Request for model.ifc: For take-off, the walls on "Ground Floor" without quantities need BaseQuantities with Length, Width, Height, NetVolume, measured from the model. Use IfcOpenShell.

First a look at what the model holds.

```python
import ifcopenshell
import ifcopenshell.util.element
import ifcopenshell.util.unit

model = ifcopenshell.open("model.ifc")
print(model.schema)
for unit_type in ("LENGTHUNIT", "AREAUNIT", "VOLUMEUNIT"):
    print(unit_type, ifcopenshell.util.unit.calculate_unit_scale(model, unit_type))
storey = next(s for s in model.by_type("IfcBuildingStorey") if s.Name == "Ground Floor")
walls = [e for e in ifcopenshell.util.element.get_decomposition(storey) if e.is_a("IfcWall")]
for e in sorted(walls, key=lambda e: e.id()):
    print(e.id(), e.is_a(), e.Name, list(ifcopenshell.util.element.get_psets(e, qtos_only=True)), sep=" | ")
```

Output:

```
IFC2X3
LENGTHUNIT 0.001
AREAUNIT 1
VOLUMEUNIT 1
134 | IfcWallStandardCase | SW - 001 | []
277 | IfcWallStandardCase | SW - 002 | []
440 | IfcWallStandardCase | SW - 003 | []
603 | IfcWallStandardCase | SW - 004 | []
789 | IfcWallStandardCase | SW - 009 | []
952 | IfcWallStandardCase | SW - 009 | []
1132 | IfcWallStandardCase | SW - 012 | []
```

```python
import ifcopenshell
import ifcopenshell.api.pset
import ifcopenshell.geom
import ifcopenshell.util.element
import ifcopenshell.util.shape
import ifcopenshell.util.unit

model = ifcopenshell.open("model.ifc")
unit_scale = ifcopenshell.util.unit.calculate_unit_scale(model)
volume_scale = ifcopenshell.util.unit.calculate_unit_scale(model, "VOLUMEUNIT")
settings = ifcopenshell.geom.settings()

storey = next(s for s in model.by_type("IfcBuildingStorey") if s.Name == "Ground Floor")
walls = [e for e in ifcopenshell.util.element.get_decomposition(storey) if e.is_a("IfcWall")]

for e in sorted(walls, key=lambda e: e.id()):
    if ifcopenshell.util.element.get_psets(e, qtos_only=True, should_inherit=False):
        continue
    # Geometry comes back in metres, in the element's own axes.
    shape = ifcopenshell.geom.create_shape(settings, e)
    values = {
        "Length": ifcopenshell.util.shape.get_x(shape.geometry) / unit_scale,
        "Width": ifcopenshell.util.shape.get_y(shape.geometry) / unit_scale,
        "Height": ifcopenshell.util.shape.get_z(shape.geometry) / unit_scale,
        "NetVolume": ifcopenshell.util.shape.get_volume(shape.geometry) / volume_scale,
    }
    qto = ifcopenshell.api.pset.add_qto(model, product=e, name="BaseQuantities")
    ifcopenshell.api.pset.edit_qto(model, qto=qto, properties=values)
    print(e.id(), {k: round(v, 3) for k, v in values.items()})

model.write("model_v2.ifc")
```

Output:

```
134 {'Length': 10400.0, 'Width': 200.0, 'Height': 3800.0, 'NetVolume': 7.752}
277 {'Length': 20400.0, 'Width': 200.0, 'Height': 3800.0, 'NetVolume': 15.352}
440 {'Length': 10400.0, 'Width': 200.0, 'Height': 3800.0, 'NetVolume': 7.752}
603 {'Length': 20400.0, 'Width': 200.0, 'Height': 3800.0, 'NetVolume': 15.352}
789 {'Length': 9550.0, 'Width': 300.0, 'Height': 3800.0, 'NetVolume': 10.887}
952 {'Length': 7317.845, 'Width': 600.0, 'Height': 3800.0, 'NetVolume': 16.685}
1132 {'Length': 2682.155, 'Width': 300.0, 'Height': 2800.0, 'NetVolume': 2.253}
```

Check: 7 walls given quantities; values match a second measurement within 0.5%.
